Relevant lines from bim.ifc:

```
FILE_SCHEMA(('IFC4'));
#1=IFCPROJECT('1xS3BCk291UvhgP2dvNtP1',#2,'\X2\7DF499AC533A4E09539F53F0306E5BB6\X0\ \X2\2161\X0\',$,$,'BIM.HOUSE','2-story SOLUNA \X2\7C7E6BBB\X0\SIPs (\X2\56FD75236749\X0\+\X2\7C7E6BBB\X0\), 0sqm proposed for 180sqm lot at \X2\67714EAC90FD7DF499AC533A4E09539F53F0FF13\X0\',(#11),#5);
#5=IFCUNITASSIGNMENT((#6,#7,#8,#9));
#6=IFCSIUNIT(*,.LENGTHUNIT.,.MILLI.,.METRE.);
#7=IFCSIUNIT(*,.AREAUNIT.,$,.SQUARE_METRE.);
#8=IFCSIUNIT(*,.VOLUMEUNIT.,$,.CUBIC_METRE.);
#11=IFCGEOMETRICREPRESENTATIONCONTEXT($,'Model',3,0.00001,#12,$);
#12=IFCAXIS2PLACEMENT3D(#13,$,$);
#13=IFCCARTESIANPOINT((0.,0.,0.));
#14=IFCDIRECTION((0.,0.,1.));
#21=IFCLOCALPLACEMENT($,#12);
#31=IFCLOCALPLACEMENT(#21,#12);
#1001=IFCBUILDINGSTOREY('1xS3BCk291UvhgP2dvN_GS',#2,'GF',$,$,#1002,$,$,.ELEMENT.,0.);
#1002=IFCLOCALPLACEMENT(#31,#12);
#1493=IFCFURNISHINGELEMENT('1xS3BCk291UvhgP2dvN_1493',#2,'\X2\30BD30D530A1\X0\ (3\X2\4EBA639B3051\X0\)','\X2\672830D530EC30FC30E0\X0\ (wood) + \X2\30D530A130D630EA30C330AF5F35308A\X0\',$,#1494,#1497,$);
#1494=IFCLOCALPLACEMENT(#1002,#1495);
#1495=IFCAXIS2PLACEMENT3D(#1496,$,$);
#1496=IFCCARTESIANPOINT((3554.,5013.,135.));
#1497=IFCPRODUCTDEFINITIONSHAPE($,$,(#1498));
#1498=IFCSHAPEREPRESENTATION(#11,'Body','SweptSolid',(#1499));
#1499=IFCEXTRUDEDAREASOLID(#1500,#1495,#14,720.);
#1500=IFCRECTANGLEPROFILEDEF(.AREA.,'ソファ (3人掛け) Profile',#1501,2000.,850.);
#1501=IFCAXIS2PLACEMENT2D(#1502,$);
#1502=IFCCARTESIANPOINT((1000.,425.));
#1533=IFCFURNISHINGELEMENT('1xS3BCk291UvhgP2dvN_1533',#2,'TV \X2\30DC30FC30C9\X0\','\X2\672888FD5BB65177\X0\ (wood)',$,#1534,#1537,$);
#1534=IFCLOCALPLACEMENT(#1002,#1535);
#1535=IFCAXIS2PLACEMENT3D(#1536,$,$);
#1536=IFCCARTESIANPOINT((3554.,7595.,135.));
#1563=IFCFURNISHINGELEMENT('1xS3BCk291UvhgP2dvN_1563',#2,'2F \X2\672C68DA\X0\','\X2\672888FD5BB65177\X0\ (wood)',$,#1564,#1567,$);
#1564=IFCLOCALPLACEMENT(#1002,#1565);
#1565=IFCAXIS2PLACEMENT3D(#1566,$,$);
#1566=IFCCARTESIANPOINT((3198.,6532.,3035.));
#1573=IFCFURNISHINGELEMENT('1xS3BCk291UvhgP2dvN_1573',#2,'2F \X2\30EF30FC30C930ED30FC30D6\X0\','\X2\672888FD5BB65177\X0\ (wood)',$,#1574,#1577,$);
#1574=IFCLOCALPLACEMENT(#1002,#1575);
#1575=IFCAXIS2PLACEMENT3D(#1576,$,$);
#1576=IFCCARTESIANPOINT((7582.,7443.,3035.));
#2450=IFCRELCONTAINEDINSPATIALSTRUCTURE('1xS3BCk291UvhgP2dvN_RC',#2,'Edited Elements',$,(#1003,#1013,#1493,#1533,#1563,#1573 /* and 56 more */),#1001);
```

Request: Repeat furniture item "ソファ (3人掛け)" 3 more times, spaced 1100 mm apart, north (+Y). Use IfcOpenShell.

```python
import numpy as np
import ifcopenshell
import ifcopenshell.api.geometry
import ifcopenshell.api.root
import ifcopenshell.util.element
import ifcopenshell.util.placement

model = ifcopenshell.open("bim.ifc")


def reuse_history(source, copy):
    """copy_class also copies each property set's owner history, people and application; keep the originals."""
    for rel in copy.IsDefinedBy:
        if rel.is_a("IfcRelDefinesByProperties") and (history := rel.RelatingPropertyDefinition.OwnerHistory):
            rel.RelatingPropertyDefinition.OwnerHistory = source.OwnerHistory
            ifcopenshell.util.element.remove_deep2(model, history)


source = model.by_id(1493)
base = ifcopenshell.util.placement.get_local_placement(source.ObjectPlacement)
step = np.array([0.0, 1.0, 0.0]) * 1100.0

for i in range(1, 4):
    copy = ifcopenshell.api.root.copy_class(model, product=source)
    copy.Representation = ifcopenshell.util.element.copy_deep(
        model, source.Representation, exclude=["IfcGeometricRepresentationContext", "IfcRepresentationMap"]
    )
    reuse_history(source, copy)
    matrix = base.copy()
    matrix[:3, 3] += i * step
    print("added at", matrix[:3, 3].round(3) + 0.0)
    ifcopenshell.api.geometry.edit_object_placement(model, product=copy, matrix=matrix, is_si=False)

model.write("bim_rev.ifc")
```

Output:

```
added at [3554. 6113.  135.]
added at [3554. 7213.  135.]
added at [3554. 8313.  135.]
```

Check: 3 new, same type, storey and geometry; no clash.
